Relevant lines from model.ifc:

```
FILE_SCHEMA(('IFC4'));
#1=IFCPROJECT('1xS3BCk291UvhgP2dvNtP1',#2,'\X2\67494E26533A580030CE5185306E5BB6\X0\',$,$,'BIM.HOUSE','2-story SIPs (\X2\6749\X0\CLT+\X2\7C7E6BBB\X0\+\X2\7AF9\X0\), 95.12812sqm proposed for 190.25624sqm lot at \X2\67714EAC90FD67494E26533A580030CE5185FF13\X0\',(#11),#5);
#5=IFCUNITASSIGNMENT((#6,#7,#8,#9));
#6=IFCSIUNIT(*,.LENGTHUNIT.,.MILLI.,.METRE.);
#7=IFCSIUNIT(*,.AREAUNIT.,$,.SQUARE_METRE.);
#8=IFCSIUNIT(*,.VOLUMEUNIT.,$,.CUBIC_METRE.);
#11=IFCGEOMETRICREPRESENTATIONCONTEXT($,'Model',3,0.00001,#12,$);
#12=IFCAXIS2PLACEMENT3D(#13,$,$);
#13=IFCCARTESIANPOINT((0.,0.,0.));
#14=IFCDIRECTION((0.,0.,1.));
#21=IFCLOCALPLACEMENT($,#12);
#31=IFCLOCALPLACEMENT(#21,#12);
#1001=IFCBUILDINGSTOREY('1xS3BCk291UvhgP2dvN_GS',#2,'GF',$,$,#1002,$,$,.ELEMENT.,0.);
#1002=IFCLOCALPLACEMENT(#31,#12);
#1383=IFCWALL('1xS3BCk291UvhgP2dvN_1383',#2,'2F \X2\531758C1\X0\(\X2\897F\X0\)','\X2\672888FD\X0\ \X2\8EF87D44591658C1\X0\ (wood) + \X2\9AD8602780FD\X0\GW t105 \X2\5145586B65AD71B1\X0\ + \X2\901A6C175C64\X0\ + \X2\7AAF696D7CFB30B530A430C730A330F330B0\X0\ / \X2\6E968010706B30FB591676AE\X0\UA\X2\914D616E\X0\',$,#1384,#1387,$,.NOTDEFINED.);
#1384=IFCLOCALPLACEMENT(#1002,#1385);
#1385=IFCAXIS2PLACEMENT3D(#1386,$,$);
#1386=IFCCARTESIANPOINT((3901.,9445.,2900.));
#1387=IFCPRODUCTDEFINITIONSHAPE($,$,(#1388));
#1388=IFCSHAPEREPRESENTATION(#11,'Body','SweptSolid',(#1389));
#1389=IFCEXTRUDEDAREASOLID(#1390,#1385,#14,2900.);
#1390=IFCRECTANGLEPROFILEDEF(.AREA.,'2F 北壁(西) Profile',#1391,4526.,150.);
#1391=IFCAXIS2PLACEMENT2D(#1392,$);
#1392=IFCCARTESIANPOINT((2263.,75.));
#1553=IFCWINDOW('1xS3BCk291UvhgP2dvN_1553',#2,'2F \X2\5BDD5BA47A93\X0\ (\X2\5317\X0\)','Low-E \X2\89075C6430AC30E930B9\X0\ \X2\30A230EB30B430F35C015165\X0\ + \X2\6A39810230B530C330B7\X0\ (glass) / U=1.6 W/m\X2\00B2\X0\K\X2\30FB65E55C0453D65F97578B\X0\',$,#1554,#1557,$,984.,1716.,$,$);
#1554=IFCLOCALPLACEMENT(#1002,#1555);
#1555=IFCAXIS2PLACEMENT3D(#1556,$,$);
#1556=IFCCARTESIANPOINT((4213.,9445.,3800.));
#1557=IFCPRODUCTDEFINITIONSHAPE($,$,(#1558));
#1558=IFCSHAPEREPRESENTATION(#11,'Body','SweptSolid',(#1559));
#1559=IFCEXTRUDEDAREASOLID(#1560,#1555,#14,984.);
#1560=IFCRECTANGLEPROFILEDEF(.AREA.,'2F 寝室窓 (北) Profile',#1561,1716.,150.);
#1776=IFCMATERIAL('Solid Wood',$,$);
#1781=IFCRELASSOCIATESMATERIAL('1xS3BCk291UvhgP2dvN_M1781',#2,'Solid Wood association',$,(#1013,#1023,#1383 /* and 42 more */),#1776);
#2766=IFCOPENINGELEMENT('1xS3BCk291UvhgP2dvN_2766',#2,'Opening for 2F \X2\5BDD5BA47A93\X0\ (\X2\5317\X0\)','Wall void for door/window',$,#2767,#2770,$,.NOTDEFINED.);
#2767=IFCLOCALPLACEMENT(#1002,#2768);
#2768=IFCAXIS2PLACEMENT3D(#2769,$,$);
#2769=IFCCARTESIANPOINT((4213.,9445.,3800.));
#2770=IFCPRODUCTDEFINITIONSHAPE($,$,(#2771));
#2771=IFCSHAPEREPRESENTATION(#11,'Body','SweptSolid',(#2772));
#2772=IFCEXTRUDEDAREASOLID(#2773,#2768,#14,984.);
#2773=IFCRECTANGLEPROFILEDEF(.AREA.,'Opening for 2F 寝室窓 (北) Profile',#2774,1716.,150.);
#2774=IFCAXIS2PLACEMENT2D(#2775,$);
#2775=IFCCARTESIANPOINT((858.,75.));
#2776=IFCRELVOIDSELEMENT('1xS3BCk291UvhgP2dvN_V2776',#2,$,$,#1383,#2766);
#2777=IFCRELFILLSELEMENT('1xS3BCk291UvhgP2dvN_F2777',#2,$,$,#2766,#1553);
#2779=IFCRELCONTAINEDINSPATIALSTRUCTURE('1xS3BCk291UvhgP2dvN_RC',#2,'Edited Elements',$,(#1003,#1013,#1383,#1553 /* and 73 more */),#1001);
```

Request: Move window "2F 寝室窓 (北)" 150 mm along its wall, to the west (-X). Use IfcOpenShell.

```python
import ifcopenshell
import ifcopenshell.api.geometry
import ifcopenshell.util.placement
import ifcopenshell.util.unit

model = ifcopenshell.open("model.ifc")
unit_scale = ifcopenshell.util.unit.calculate_unit_scale(model)

window = model.by_guid("1xS3BCk291UvhgP2dvN_1553")
opening = window.FillsVoids[0].RelatingOpeningElement
wall = opening.VoidsElements[0].RelatingBuildingElement

wall_matrix = ifcopenshell.util.placement.get_local_placement(wall.ObjectPlacement)
shift = wall_matrix[:3, 0] * -0.15 / unit_scale
before = ifcopenshell.util.placement.get_local_placement(window.ObjectPlacement)[:3, 3].copy()

# The window is not placed relative to its opening, so move both.
for product in (opening, window):
    matrix = ifcopenshell.util.placement.get_local_placement(product.ObjectPlacement)
    matrix[:3, 3] += shift
    ifcopenshell.api.geometry.edit_object_placement(model, product=product, matrix=matrix, is_si=False)

after = ifcopenshell.util.placement.get_local_placement(window.ObjectPlacement)[:3, 3]
print("window moved by", (after - before).round(3) + 0.0)

model.write("model_edited.ifc")
```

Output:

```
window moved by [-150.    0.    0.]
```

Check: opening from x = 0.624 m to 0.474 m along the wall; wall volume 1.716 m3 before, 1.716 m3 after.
